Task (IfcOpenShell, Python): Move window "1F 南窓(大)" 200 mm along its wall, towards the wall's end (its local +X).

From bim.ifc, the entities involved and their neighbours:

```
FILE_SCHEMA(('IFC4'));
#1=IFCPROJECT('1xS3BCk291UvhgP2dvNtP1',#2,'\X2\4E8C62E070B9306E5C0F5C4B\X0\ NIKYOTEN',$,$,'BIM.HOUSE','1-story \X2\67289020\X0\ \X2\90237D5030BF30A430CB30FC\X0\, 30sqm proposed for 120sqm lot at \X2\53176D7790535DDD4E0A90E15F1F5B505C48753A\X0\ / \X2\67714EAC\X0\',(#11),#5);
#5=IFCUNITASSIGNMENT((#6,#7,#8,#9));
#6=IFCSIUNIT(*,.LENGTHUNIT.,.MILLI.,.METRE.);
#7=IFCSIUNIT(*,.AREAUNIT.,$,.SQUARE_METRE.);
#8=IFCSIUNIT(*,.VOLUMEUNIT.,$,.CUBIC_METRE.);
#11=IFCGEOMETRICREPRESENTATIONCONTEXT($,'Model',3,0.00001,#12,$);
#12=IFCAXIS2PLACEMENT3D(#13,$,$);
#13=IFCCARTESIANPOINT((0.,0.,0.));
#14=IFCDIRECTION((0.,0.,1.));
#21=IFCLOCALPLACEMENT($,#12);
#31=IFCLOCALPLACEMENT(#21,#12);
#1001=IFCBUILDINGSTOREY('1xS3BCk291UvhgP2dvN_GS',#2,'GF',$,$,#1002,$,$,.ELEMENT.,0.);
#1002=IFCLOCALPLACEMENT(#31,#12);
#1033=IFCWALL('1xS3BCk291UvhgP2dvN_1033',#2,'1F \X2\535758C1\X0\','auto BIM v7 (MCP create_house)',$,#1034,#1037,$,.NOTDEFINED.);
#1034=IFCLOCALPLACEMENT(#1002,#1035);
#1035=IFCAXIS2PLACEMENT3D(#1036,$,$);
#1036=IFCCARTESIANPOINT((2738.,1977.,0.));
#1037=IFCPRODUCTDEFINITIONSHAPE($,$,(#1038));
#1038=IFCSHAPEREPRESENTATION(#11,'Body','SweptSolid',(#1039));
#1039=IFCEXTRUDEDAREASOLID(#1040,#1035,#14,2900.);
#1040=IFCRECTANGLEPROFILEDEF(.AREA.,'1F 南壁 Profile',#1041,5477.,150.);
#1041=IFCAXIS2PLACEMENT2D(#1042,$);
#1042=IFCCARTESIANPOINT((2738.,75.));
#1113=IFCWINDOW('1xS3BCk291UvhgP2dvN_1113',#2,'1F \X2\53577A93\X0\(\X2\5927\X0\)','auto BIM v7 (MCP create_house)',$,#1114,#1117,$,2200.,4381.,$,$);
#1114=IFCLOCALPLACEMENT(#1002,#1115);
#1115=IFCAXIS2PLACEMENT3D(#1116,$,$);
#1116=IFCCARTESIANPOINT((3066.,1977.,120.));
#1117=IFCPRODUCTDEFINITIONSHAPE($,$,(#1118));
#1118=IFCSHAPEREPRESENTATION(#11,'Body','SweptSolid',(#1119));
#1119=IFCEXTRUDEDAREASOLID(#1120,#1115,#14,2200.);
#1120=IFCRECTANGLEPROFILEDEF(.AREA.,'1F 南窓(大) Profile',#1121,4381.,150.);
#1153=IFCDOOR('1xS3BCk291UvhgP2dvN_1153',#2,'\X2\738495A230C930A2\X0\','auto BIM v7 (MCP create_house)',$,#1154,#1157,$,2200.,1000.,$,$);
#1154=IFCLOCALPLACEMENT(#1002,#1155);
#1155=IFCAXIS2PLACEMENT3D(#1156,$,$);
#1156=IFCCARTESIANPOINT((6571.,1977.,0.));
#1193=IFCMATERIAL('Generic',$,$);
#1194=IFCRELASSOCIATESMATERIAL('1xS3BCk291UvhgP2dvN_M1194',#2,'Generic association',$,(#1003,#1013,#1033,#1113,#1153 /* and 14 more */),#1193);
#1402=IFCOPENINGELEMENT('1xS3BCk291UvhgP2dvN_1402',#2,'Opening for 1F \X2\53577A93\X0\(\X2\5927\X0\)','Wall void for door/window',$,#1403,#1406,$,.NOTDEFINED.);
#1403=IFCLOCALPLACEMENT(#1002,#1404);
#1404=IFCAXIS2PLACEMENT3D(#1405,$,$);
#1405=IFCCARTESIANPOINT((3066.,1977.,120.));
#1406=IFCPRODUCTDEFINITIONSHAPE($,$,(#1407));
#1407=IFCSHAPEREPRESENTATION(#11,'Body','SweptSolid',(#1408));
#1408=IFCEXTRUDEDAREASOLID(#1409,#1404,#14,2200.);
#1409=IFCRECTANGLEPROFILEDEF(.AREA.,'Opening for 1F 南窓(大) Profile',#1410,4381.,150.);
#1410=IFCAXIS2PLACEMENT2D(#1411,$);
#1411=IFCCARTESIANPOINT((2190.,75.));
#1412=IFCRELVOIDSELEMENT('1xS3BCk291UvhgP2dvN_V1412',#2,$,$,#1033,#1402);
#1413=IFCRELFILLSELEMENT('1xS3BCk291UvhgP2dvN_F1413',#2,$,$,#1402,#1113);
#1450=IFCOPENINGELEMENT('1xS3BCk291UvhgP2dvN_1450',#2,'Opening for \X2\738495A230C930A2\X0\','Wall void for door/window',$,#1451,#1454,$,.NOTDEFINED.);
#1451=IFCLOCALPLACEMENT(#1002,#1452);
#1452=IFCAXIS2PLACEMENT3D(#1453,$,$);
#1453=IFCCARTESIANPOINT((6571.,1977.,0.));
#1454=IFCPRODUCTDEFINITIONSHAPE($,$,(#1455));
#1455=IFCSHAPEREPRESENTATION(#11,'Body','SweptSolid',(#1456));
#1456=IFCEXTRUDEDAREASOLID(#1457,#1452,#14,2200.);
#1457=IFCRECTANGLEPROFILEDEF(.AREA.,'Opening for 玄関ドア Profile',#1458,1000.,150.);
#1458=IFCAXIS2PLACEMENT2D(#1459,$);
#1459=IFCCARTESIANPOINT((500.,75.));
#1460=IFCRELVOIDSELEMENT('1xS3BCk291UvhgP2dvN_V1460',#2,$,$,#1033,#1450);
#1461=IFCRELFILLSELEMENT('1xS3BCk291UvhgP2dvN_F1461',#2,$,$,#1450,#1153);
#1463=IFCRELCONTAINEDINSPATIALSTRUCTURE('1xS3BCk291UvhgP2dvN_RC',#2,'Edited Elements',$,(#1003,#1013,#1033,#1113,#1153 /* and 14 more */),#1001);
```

```python
import ifcopenshell
import ifcopenshell.api.geometry
import ifcopenshell.util.placement
import ifcopenshell.util.unit

model = ifcopenshell.open("bim.ifc")
unit_scale = ifcopenshell.util.unit.calculate_unit_scale(model)

window = model.by_guid("1xS3BCk291UvhgP2dvN_1113")
opening = window.FillsVoids[0].RelatingOpeningElement
wall = opening.VoidsElements[0].RelatingBuildingElement

wall_matrix = ifcopenshell.util.placement.get_local_placement(wall.ObjectPlacement)
shift = wall_matrix[:3, 0] * 0.2 / unit_scale
before = ifcopenshell.util.placement.get_local_placement(window.ObjectPlacement)[:3, 3].copy()

# The window is not placed relative to its opening, so move both.
for product in (opening, window):
    matrix = ifcopenshell.util.placement.get_local_placement(product.ObjectPlacement)
    matrix[:3, 3] += shift
    ifcopenshell.api.geometry.edit_object_placement(model, product=product, matrix=matrix, is_si=False)

after = ifcopenshell.util.placement.get_local_placement(window.ObjectPlacement)[:3, 3]
print("window moved by", (after - before).round(3) + 0.0)

model.write("bim_rev.ifc")
```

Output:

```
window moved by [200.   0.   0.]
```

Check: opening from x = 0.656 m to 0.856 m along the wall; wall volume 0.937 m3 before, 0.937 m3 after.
